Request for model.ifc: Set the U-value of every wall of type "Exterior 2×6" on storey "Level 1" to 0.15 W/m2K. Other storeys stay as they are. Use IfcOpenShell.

First a look at what the model holds.

```python
import ifcopenshell
import ifcopenshell.util.element

model = ifcopenshell.open("model.ifc")
print(model.schema)
storey = next(s for s in model.by_type("IfcBuildingStorey") if s.Name == "Level 1")
walls = [e for e in ifcopenshell.util.element.get_decomposition(storey) if e.is_a("IfcWall")]
seen = {}
for e in walls:
    element_type = ifcopenshell.util.element.get_type(e)
    key = (element_type.Name if element_type != e and element_type else None, ifcopenshell.util.element.get_pset(e, "Pset_WallCommon", "ThermalTransmittance"))
    seen[key] = seen.get(key, 0) + 1
for (name, value), count in sorted(seen.items(), key=str):
    print(count, "x", name, "|", value)
```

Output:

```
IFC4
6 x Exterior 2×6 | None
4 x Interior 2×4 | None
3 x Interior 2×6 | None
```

```python
import ifcopenshell
import ifcopenshell.api.pset
import ifcopenshell.util.element

model = ifcopenshell.open("model.ifc")

storey = next(s for s in model.by_type("IfcBuildingStorey") if s.Name == "Level 1")
walls = [e for e in ifcopenshell.util.element.get_decomposition(storey) if e.is_a("IfcWall")]

count = 0
for e in walls:
    element_type = ifcopenshell.util.element.get_type(e)
    if element_type in (None, e) or element_type.Name != "Exterior 2×6":
        continue
    # add_pset returns the element's existing set when there is one.
    pset = ifcopenshell.api.pset.add_pset(model, product=e, name="Pset_WallCommon")
    ifcopenshell.api.pset.edit_pset(model, pset=pset, properties={"ThermalTransmittance": 0.15})
    count += 1

print(count, "walls updated")

model.write("model_v2.ifc")
```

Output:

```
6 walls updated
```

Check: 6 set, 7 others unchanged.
